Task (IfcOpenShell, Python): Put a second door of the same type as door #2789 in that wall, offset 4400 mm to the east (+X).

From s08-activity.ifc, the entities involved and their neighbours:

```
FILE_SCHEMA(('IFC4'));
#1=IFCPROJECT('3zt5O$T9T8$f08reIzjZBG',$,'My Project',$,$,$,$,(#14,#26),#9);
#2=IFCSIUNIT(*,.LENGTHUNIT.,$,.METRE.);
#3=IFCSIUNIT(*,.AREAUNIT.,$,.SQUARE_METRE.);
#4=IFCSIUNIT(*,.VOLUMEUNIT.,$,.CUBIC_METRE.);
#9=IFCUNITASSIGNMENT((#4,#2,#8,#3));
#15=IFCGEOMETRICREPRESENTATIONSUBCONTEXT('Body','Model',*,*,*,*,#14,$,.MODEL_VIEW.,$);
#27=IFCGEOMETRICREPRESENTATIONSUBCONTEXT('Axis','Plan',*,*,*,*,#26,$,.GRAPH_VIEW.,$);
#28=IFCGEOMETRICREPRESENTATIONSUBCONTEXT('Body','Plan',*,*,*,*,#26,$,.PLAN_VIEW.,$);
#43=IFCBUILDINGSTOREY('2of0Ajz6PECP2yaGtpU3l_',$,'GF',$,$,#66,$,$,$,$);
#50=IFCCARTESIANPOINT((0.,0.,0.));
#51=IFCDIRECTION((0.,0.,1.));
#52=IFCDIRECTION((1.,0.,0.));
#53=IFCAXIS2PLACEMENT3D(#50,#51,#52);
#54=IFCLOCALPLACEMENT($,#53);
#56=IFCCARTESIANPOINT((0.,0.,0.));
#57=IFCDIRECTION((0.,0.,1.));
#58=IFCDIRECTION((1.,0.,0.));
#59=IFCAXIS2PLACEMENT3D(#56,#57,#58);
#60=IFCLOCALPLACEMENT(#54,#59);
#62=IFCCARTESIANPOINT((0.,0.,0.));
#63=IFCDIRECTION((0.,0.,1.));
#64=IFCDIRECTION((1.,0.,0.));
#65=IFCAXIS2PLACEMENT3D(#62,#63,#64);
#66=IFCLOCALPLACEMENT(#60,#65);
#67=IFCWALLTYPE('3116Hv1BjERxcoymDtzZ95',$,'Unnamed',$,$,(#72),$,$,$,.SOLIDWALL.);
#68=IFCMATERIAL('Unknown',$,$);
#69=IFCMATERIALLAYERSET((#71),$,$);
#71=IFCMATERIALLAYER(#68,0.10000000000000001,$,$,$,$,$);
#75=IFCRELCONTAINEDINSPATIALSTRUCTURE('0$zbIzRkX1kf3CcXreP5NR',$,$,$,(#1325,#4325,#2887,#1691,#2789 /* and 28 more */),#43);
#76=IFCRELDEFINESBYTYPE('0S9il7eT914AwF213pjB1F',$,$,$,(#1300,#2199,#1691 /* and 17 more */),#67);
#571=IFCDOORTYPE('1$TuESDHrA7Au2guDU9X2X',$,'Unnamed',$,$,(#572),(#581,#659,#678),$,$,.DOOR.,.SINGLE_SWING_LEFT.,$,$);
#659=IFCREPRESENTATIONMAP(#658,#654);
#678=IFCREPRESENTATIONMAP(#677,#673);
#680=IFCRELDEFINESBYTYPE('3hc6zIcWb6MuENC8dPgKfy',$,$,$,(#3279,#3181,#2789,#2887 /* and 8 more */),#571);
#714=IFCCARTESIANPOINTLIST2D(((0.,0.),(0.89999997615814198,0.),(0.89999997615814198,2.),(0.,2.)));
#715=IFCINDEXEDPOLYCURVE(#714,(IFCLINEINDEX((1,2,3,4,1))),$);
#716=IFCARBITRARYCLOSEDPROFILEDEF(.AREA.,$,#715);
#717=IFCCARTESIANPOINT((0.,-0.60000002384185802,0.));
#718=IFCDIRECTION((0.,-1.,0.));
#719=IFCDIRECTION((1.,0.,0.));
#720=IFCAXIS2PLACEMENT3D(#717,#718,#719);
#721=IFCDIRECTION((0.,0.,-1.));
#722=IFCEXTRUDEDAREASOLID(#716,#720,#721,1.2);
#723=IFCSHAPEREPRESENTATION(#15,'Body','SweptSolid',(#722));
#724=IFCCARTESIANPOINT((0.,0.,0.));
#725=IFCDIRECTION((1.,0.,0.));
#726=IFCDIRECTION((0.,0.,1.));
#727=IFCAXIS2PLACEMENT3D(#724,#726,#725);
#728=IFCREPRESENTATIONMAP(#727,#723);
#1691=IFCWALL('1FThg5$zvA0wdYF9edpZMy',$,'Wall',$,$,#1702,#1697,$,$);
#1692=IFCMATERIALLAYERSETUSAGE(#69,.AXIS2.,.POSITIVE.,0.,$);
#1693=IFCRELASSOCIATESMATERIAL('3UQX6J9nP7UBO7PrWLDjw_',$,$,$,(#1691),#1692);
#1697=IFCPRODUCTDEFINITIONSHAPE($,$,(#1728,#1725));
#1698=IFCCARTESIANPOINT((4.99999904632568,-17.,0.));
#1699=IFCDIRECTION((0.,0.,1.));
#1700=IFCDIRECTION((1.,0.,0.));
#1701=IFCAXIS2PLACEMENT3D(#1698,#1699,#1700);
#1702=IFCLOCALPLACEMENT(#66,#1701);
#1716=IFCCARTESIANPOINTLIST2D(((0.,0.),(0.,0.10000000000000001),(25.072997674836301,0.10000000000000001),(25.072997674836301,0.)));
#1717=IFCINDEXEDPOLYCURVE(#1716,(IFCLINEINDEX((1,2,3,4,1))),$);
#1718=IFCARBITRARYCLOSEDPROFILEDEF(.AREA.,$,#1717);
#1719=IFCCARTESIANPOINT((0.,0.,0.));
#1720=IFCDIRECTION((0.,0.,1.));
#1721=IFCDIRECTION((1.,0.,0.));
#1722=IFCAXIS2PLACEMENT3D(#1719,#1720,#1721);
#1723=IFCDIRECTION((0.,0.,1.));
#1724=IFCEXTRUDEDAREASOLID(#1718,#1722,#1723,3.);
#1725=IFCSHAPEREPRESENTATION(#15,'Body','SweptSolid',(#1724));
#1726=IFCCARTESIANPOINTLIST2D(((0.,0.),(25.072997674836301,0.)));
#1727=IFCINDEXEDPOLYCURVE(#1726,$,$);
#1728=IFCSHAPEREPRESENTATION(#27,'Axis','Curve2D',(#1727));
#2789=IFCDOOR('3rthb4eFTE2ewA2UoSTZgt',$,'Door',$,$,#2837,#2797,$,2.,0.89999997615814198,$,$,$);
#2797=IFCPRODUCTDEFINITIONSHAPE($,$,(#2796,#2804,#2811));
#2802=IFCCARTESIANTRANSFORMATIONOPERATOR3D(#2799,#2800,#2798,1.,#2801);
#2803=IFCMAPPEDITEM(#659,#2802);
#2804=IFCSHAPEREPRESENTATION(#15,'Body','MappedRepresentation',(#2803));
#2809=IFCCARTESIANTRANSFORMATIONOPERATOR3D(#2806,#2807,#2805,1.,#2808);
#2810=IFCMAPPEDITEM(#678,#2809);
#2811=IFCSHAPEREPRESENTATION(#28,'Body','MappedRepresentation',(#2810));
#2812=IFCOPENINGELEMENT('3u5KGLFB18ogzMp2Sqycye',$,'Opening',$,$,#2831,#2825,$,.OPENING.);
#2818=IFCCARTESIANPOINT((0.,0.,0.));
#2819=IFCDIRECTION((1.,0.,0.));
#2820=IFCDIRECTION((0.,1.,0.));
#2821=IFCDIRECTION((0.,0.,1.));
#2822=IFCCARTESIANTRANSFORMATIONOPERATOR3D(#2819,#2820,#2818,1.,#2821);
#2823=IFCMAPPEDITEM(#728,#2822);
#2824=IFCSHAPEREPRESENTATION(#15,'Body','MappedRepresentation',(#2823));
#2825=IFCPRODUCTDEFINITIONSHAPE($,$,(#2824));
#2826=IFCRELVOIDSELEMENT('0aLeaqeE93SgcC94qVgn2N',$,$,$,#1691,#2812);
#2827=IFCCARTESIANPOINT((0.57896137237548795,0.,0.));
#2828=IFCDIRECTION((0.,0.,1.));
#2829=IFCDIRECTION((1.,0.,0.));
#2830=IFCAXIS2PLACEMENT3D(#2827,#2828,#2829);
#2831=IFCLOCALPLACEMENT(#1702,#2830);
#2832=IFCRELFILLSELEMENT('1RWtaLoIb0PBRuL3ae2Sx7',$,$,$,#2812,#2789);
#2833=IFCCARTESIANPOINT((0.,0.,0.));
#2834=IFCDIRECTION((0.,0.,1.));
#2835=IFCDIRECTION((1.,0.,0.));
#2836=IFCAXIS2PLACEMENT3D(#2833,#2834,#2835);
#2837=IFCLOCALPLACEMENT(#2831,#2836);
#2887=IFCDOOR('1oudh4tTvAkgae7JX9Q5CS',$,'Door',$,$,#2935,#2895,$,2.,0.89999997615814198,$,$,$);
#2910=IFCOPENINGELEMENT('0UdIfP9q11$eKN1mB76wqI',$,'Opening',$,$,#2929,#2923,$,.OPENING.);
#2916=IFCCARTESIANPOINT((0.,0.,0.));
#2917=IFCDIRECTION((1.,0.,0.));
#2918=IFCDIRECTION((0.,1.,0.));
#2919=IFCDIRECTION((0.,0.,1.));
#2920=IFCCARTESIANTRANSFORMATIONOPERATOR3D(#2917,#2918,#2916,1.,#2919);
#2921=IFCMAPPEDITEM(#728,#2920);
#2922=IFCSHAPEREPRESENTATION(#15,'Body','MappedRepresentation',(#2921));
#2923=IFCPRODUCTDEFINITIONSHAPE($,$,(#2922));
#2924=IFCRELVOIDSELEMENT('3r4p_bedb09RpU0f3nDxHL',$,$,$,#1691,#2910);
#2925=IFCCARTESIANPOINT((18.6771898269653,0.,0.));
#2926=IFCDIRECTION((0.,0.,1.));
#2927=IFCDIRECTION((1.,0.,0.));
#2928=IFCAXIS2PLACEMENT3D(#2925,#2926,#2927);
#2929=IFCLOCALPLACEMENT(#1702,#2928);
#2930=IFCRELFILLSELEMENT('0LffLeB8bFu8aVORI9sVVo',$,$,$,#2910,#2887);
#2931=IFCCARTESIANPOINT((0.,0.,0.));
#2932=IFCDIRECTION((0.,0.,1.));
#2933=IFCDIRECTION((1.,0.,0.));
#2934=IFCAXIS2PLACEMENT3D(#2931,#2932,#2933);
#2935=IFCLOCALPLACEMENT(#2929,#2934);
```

```python
import ifcopenshell
import ifcopenshell.api.feature
import ifcopenshell.api.geometry
import ifcopenshell.api.root
import ifcopenshell.geom
import ifcopenshell.util.element
import ifcopenshell.util.placement
import ifcopenshell.util.shape

model = ifcopenshell.open("s08-activity.ifc")
settings = ifcopenshell.geom.settings()


def volume(element):
    """Net volume in cubic metres, openings subtracted."""
    shape = ifcopenshell.geom.create_shape(settings, element)
    return ifcopenshell.util.shape.get_volume(shape.geometry)


door = model.by_guid("3rthb4eFTE2ewA2UoSTZgt")
opening = door.FillsVoids[0].RelatingOpeningElement
wall = opening.VoidsElements[0].RelatingBuildingElement
before = volume(wall)
shift = ifcopenshell.util.placement.get_local_placement(wall.ObjectPlacement)[:3, 0] * 4.4

# copy_class copies the void relationship, type, container and properties, but no geometry.
new_opening = ifcopenshell.api.root.copy_class(model, product=opening)
new_opening.Representation = ifcopenshell.util.element.copy_deep(
    model, opening.Representation, exclude=["IfcGeometricRepresentationContext", "IfcRepresentationMap"]
)
new_door = ifcopenshell.api.root.copy_class(model, product=door)
new_door.Representation = ifcopenshell.util.element.copy_deep(
    model, door.Representation, exclude=["IfcGeometricRepresentationContext", "IfcRepresentationMap"]
)
ifcopenshell.api.feature.add_filling(model, opening=new_opening, element=new_door)

for old, new in ((opening, new_opening), (door, new_door)):
    matrix = ifcopenshell.util.placement.get_local_placement(old.ObjectPlacement)
    matrix[:3, 3] += shift
    ifcopenshell.api.geometry.edit_object_placement(model, product=new, matrix=matrix, is_si=False)

after = volume(wall)

print(f"wall volume {before:.3f} -> {after:.3f} m3")

model.write("s08-activity_edited.ifc")
```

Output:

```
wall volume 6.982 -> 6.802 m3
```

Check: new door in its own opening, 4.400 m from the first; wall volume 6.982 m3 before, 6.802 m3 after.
